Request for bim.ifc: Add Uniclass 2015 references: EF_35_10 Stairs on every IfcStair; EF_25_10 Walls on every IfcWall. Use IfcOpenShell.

First a look at what the model holds.

```python
import ifcopenshell

model = ifcopenshell.open("bim.ifc")
print(model.schema)
print("classifications:", [c.Name for c in model.by_type("IfcClassification")])
for ifc_class in ("IfcDoor", "IfcRoof", "IfcStair", "IfcWall", "IfcWindow"):
    print(ifc_class, len(model.by_type(ifc_class)))
```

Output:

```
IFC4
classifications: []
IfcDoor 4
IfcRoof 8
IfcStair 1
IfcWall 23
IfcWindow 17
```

```python
import ifcopenshell
import ifcopenshell.api.classification

model = ifcopenshell.open("bim.ifc")

system = ifcopenshell.api.classification.add_classification(model, classification="Uniclass 2015")

codes = {
    "IfcStair": ("EF_35_10", "Stairs"),
    "IfcWall": ("EF_25_10", "Walls"),
}
for ifc_class, (code, name) in codes.items():
    products = model.by_type(ifc_class)
    ifcopenshell.api.classification.add_reference(
        model, products=products, classification=system, identification=code, name=name
    )
    print(code, len(products))

model.write("bim-out.ifc")
```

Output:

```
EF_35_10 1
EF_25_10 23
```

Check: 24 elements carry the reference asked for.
